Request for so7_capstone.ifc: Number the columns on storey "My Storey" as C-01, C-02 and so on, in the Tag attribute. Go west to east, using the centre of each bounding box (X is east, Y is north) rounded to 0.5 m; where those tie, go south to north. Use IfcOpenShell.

First a look at what the model holds.

```python
import ifcopenshell
import ifcopenshell.util.element
import ifcopenshell.util.placement

model = ifcopenshell.open("so7_capstone.ifc")
print(model.schema)
storey = next(s for s in model.by_type("IfcBuildingStorey") if s.Name == "My Storey")
columns = [e for e in ifcopenshell.util.element.get_decomposition(storey) if e.is_a("IfcColumn")]
for e in sorted(columns, key=lambda e: e.id()):
    origin = ifcopenshell.util.placement.get_local_placement(e.ObjectPlacement)[:3, 3]
    print(e.id(), e.Tag, e.Name, origin.round(2) + 0.0, sep=" | ")
```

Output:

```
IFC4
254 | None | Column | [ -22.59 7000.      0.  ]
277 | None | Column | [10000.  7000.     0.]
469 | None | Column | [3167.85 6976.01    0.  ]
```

```python
import ifcopenshell
import ifcopenshell.geom
import ifcopenshell.util.element
import ifcopenshell.util.shape

model = ifcopenshell.open("so7_capstone.ifc")
settings = ifcopenshell.geom.settings()
settings.set("use-world-coords", True)


def centre(element):
    shape = ifcopenshell.geom.create_shape(settings, element)
    return ifcopenshell.util.shape.get_bbox_centroid(shape.geometry)


storey = next(s for s in model.by_type("IfcBuildingStorey") if s.Name == "My Storey")
columns = [e for e in ifcopenshell.util.element.get_decomposition(storey) if e.is_a("IfcColumn")]

# Insertion points can sit at a corner or the storey origin, so sort by the geometry (in metres).
centres = {e: centre(e) for e in columns}
columns.sort(key=lambda e: (round(centres[e][0] / 0.5), centres[e][1]))

for i, e in enumerate(columns, start=1):
    number = f"C-{i:02d}"
    e.Tag = number
    print(e.id(), number)

model.write("so7_capstone_v2.ifc")
```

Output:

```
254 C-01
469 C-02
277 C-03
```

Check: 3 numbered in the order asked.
